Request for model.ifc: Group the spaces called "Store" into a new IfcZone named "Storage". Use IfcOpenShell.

First a look at what the model holds.

```python
import ifcopenshell

model = ifcopenshell.open("model.ifc")
print(model.schema)
seen = {}
for space in model.by_type("IfcSpace"):
    seen[space.LongName] = seen.get(space.LongName, 0) + 1
for name, count in sorted(seen.items(), key=str):
    print(count, "x", name)
print("zones:", [z.Name for z in model.by_type("IfcZone")][:20])
```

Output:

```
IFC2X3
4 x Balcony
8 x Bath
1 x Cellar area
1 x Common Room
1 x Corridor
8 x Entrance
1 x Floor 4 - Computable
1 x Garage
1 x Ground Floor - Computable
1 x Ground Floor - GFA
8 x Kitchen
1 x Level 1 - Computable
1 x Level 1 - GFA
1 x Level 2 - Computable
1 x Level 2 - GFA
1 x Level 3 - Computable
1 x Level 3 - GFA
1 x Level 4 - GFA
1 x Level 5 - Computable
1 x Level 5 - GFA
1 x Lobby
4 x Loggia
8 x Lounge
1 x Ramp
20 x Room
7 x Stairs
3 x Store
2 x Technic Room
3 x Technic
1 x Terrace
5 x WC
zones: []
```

```python
import ifcopenshell
import ifcopenshell.api.group
import ifcopenshell.api.root

model = ifcopenshell.open("model.ifc")

names = {"Store"}
spaces = [s for s in model.by_type("IfcSpace") if s.LongName in names]

zone = ifcopenshell.api.root.create_entity(model, ifc_class="IfcZone", name="Storage")
ifcopenshell.api.group.assign_group(model, products=spaces, group=zone)
print(len(spaces), "spaces in", zone.Name)

model.write("model-out.ifc")
```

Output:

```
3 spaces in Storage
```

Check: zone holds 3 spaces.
